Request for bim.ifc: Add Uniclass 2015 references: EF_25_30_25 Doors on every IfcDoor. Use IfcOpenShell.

First a look at what the model holds.

```python
import ifcopenshell

model = ifcopenshell.open("bim.ifc")
print(model.schema)
print("classifications:", [c.Name for c in model.by_type("IfcClassification")])
for ifc_class in ("IfcDoor", "IfcRoof", "IfcStair", "IfcWall", "IfcWindow"):
    print(ifc_class, len(model.by_type(ifc_class)))
```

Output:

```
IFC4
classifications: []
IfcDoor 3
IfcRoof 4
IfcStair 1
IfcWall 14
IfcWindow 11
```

```python
import ifcopenshell
import ifcopenshell.api.classification

model = ifcopenshell.open("bim.ifc")

system = ifcopenshell.api.classification.add_classification(model, classification="Uniclass 2015")

codes = {
    "IfcDoor": ("EF_25_30_25", "Doors"),
}
for ifc_class, (code, name) in codes.items():
    products = model.by_type(ifc_class)
    ifcopenshell.api.classification.add_reference(
        model, products=products, classification=system, identification=code, name=name
    )
    print(code, len(products))

model.write("bim-out.ifc")
```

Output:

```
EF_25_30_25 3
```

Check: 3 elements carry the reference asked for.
